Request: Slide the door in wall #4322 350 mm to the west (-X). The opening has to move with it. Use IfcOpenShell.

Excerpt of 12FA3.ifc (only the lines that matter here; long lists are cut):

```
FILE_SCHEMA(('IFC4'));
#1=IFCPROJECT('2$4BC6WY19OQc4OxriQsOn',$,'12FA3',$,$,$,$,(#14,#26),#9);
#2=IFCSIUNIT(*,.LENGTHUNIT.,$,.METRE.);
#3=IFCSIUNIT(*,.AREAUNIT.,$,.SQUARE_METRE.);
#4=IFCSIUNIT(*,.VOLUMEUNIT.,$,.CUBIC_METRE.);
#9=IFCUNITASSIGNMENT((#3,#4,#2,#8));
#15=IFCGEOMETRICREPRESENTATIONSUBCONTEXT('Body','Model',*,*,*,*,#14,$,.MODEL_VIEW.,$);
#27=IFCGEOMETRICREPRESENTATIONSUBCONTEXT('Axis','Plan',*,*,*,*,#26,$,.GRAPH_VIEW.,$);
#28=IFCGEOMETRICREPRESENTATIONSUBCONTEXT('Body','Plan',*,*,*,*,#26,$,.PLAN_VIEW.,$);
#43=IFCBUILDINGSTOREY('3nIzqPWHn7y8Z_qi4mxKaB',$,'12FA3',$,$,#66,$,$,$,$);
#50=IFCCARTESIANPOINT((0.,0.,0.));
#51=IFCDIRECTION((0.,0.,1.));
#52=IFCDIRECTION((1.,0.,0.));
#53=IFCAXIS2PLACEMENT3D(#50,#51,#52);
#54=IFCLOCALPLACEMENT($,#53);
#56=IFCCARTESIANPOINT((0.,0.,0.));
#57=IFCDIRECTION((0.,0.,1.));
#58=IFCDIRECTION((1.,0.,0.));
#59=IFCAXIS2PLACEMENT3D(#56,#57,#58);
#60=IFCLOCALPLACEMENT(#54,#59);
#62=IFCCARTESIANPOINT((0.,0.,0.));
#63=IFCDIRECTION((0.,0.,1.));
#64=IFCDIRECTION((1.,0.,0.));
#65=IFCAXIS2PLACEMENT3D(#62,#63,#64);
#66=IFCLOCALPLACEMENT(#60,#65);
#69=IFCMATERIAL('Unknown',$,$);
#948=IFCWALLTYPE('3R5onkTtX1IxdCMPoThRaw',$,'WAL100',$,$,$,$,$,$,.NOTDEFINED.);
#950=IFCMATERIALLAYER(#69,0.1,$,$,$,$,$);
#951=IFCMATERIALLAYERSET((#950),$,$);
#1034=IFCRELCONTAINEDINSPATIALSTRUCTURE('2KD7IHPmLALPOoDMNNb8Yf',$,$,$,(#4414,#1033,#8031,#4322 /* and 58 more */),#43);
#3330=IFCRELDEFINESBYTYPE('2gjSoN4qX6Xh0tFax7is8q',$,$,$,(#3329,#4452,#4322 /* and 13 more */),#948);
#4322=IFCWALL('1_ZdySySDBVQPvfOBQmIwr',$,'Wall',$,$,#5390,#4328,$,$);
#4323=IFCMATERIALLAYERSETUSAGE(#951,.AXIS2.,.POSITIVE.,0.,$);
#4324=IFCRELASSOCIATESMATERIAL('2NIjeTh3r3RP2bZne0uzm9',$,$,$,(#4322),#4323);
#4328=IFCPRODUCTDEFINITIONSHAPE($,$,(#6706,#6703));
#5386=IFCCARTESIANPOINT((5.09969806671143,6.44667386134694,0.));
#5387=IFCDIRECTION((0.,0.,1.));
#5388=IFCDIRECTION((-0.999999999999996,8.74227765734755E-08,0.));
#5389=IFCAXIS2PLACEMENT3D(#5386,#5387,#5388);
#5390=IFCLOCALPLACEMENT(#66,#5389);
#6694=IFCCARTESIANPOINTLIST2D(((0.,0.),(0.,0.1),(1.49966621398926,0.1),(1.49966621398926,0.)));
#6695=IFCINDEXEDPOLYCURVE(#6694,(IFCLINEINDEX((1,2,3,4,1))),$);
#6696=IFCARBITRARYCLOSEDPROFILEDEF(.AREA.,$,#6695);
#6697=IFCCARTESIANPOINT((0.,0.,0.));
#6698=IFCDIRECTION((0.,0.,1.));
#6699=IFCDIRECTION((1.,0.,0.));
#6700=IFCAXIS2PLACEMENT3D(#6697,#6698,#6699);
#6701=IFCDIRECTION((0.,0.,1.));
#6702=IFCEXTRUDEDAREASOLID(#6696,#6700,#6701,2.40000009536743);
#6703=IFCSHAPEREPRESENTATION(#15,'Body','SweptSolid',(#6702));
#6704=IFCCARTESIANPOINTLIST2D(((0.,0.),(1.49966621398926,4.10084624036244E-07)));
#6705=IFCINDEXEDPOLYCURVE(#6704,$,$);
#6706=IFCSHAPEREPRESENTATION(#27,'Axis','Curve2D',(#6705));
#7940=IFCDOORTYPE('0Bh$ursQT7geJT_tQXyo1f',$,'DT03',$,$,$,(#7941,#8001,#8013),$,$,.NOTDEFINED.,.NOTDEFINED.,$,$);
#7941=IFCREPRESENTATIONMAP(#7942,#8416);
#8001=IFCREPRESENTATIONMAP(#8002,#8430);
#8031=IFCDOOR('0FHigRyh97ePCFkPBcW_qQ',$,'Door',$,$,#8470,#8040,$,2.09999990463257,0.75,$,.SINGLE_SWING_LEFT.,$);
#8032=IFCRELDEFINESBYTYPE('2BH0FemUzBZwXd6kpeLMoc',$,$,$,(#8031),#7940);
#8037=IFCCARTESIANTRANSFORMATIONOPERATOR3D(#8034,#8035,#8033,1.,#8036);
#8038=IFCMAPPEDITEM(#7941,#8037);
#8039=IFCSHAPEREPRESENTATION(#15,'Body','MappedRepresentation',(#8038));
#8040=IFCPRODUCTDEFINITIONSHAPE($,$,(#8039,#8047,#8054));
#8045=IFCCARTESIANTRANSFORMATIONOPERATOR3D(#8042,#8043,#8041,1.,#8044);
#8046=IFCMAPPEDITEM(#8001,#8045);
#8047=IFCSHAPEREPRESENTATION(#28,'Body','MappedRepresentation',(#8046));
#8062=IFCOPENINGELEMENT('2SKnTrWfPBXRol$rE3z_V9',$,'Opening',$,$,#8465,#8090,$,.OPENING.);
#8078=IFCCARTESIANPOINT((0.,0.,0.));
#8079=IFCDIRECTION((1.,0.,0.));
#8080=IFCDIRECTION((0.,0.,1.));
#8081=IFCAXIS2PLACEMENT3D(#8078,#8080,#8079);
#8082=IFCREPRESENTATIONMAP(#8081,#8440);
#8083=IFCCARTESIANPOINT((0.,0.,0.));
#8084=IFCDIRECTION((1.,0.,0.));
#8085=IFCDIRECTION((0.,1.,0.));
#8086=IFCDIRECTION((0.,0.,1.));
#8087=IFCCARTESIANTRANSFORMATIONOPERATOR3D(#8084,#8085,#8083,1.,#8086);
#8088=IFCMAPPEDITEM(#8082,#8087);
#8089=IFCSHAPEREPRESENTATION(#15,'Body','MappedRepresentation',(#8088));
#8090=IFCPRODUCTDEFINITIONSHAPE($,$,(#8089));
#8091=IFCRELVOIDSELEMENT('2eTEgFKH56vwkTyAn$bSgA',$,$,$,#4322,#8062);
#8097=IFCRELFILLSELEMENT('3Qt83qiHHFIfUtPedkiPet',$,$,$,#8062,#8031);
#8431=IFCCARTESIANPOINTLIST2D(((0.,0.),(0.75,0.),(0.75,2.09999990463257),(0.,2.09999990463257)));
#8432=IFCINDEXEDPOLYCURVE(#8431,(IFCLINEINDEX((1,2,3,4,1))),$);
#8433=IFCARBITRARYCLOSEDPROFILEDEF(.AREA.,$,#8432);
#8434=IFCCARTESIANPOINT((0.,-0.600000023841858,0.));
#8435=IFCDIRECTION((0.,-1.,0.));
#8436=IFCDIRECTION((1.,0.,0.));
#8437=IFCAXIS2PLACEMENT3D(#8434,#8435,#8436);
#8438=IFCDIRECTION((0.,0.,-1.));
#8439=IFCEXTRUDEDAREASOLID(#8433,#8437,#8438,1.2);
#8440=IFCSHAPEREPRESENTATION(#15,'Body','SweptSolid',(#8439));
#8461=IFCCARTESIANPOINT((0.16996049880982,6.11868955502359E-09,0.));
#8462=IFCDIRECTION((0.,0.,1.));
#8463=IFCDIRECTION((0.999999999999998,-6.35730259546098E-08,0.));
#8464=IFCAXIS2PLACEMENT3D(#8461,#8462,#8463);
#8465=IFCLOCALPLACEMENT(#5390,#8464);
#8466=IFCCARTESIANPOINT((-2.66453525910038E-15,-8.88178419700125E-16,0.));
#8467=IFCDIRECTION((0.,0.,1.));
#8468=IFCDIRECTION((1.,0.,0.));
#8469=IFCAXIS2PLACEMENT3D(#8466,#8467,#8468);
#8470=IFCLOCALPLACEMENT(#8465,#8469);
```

```python
import ifcopenshell
import ifcopenshell.api.geometry
import ifcopenshell.util.placement
import ifcopenshell.util.unit

model = ifcopenshell.open("12FA3.ifc")
unit_scale = ifcopenshell.util.unit.calculate_unit_scale(model)

door = model.by_id(8031)
opening = door.FillsVoids[0].RelatingOpeningElement
wall = opening.VoidsElements[0].RelatingBuildingElement

wall_matrix = ifcopenshell.util.placement.get_local_placement(wall.ObjectPlacement)
shift = wall_matrix[:3, 0] * 0.35 / unit_scale
before = ifcopenshell.util.placement.get_local_placement(door.ObjectPlacement)[:3, 3].copy()

# The door is placed relative to its opening, so it follows when the opening moves.
matrix = ifcopenshell.util.placement.get_local_placement(opening.ObjectPlacement)
matrix[:3, 3] += shift
ifcopenshell.api.geometry.edit_object_placement(
    model, product=opening, matrix=matrix, is_si=False, should_transform_children=True
)

after = ifcopenshell.util.placement.get_local_placement(door.ObjectPlacement)[:3, 3]
print("door moved by", (after - before).round(3) + 0.0)

model.write("12FA3-out.ifc")
```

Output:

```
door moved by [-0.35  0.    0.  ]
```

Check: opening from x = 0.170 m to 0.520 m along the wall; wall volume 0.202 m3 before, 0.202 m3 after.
